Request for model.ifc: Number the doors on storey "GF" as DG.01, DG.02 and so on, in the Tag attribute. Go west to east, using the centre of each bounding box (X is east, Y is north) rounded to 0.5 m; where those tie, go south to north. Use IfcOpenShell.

First a look at what the model holds.

```python
import ifcopenshell
import ifcopenshell.util.element
import ifcopenshell.util.placement

model = ifcopenshell.open("model.ifc")
print(model.schema)
storey = next(s for s in model.by_type("IfcBuildingStorey") if s.Name == "GF")
doors = [e for e in ifcopenshell.util.element.get_decomposition(storey) if e.is_a("IfcDoor")]
for e in sorted(doors, key=lambda e: e.id()):
    origin = ifcopenshell.util.placement.get_local_placement(e.ObjectPlacement)[:3, 3]
    print(e.id(), e.Tag, e.Name, origin.round(2) + 0.0, sep=" | ")
```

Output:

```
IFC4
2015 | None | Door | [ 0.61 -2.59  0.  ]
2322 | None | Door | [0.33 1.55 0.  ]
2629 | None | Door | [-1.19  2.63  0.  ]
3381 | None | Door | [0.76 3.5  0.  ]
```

```python
import ifcopenshell
import ifcopenshell.geom
import ifcopenshell.util.element
import ifcopenshell.util.shape

model = ifcopenshell.open("model.ifc")
settings = ifcopenshell.geom.settings()
settings.set("use-world-coords", True)


def centre(element):
    shape = ifcopenshell.geom.create_shape(settings, element)
    return ifcopenshell.util.shape.get_bbox_centroid(shape.geometry)


storey = next(s for s in model.by_type("IfcBuildingStorey") if s.Name == "GF")
doors = [e for e in ifcopenshell.util.element.get_decomposition(storey) if e.is_a("IfcDoor")]

# Insertion points can sit at a corner or the storey origin, so sort by the geometry (in metres).
centres = {e: centre(e) for e in doors}
doors.sort(key=lambda e: (round(centres[e][0] / 0.5), centres[e][1]))

for i, e in enumerate(doors, start=1):
    number = f"DG.{i:02d}"
    e.Tag = number
    print(e.id(), number)

model.write("model_v2.ifc")
```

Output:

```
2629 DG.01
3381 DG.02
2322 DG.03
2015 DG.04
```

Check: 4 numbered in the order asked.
